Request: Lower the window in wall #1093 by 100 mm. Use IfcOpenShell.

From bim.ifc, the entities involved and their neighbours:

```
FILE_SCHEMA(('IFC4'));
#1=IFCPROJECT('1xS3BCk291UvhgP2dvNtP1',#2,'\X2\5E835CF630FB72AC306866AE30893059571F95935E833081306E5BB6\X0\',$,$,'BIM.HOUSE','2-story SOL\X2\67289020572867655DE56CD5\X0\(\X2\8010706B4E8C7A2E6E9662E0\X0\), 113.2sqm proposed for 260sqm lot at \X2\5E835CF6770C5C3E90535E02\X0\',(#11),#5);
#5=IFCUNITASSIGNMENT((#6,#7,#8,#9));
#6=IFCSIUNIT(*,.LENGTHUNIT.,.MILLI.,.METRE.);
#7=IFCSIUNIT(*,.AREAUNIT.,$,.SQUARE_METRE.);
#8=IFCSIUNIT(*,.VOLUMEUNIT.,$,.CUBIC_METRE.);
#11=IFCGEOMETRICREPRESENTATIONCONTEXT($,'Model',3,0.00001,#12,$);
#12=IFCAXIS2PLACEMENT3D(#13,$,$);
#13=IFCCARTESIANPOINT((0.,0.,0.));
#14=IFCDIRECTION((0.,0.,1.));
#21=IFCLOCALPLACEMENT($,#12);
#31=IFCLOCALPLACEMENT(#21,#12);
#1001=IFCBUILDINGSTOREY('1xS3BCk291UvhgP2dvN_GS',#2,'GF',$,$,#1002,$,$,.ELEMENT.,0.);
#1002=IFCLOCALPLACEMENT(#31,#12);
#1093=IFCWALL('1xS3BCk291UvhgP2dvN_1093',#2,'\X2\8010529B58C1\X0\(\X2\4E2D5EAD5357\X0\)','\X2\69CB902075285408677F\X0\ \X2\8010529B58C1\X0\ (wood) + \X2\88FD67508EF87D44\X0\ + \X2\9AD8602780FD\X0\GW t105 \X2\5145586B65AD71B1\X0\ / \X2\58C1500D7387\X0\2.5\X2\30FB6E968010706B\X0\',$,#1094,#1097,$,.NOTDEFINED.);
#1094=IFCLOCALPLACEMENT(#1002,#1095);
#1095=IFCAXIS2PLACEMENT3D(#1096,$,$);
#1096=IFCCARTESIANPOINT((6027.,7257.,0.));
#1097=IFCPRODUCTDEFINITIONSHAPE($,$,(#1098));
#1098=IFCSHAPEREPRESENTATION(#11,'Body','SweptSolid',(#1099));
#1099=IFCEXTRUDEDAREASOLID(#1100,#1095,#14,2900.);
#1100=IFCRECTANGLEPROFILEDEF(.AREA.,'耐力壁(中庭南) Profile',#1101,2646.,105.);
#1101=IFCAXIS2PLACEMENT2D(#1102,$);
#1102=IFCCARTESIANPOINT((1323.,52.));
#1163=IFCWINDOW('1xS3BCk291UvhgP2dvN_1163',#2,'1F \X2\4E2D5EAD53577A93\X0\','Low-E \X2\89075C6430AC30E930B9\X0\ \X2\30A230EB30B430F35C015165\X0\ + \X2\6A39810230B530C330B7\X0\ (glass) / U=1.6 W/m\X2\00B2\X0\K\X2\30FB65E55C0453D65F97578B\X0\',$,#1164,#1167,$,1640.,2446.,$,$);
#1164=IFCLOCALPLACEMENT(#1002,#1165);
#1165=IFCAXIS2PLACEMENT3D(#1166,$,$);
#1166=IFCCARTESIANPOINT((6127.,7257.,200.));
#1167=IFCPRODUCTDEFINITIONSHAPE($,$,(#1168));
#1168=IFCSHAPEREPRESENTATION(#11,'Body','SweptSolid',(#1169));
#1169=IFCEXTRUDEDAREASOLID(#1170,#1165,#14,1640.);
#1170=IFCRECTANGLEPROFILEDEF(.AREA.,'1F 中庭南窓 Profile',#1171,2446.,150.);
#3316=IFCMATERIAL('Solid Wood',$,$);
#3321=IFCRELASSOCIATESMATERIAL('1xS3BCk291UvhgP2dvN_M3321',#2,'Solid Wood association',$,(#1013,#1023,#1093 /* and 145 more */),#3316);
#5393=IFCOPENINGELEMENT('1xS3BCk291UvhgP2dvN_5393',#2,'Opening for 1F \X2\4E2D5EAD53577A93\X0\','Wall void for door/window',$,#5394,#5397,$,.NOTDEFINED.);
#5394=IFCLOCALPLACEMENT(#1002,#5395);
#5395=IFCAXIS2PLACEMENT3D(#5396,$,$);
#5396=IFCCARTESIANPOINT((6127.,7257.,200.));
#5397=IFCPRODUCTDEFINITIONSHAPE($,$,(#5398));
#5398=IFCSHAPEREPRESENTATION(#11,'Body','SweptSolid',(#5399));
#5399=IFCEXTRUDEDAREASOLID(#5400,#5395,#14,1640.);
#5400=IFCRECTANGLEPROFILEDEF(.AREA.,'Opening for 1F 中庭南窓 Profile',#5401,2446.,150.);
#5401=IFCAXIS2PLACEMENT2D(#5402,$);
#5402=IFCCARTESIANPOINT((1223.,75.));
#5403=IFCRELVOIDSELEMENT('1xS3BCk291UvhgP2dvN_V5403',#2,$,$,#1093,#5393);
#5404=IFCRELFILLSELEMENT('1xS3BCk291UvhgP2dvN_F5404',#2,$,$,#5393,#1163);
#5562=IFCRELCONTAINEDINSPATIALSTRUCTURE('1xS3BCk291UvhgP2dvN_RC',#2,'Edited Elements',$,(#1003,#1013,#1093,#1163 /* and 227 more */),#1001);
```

```python
import numpy as np
import ifcopenshell
import ifcopenshell.api.geometry
import ifcopenshell.util.placement
import ifcopenshell.util.unit

model = ifcopenshell.open("bim.ifc")
unit_scale = ifcopenshell.util.unit.calculate_unit_scale(model)

window = model.by_guid("1xS3BCk291UvhgP2dvN_1163")
opening = window.FillsVoids[0].RelatingOpeningElement
dz = -0.1 / unit_scale

shift = np.array([0.0, 0.0, dz])
# The window is not placed relative to its opening, so move both.
for product in (opening, window):
    matrix = ifcopenshell.util.placement.get_local_placement(product.ObjectPlacement)
    matrix[:3, 3] += shift
    ifcopenshell.api.geometry.edit_object_placement(model, product=product, matrix=matrix, is_si=False)

print(f"moved by {dz * unit_scale:+.3f} m")

model.write("bim_v2.ifc")
```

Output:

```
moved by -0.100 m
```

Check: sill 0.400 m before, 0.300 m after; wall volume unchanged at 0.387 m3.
